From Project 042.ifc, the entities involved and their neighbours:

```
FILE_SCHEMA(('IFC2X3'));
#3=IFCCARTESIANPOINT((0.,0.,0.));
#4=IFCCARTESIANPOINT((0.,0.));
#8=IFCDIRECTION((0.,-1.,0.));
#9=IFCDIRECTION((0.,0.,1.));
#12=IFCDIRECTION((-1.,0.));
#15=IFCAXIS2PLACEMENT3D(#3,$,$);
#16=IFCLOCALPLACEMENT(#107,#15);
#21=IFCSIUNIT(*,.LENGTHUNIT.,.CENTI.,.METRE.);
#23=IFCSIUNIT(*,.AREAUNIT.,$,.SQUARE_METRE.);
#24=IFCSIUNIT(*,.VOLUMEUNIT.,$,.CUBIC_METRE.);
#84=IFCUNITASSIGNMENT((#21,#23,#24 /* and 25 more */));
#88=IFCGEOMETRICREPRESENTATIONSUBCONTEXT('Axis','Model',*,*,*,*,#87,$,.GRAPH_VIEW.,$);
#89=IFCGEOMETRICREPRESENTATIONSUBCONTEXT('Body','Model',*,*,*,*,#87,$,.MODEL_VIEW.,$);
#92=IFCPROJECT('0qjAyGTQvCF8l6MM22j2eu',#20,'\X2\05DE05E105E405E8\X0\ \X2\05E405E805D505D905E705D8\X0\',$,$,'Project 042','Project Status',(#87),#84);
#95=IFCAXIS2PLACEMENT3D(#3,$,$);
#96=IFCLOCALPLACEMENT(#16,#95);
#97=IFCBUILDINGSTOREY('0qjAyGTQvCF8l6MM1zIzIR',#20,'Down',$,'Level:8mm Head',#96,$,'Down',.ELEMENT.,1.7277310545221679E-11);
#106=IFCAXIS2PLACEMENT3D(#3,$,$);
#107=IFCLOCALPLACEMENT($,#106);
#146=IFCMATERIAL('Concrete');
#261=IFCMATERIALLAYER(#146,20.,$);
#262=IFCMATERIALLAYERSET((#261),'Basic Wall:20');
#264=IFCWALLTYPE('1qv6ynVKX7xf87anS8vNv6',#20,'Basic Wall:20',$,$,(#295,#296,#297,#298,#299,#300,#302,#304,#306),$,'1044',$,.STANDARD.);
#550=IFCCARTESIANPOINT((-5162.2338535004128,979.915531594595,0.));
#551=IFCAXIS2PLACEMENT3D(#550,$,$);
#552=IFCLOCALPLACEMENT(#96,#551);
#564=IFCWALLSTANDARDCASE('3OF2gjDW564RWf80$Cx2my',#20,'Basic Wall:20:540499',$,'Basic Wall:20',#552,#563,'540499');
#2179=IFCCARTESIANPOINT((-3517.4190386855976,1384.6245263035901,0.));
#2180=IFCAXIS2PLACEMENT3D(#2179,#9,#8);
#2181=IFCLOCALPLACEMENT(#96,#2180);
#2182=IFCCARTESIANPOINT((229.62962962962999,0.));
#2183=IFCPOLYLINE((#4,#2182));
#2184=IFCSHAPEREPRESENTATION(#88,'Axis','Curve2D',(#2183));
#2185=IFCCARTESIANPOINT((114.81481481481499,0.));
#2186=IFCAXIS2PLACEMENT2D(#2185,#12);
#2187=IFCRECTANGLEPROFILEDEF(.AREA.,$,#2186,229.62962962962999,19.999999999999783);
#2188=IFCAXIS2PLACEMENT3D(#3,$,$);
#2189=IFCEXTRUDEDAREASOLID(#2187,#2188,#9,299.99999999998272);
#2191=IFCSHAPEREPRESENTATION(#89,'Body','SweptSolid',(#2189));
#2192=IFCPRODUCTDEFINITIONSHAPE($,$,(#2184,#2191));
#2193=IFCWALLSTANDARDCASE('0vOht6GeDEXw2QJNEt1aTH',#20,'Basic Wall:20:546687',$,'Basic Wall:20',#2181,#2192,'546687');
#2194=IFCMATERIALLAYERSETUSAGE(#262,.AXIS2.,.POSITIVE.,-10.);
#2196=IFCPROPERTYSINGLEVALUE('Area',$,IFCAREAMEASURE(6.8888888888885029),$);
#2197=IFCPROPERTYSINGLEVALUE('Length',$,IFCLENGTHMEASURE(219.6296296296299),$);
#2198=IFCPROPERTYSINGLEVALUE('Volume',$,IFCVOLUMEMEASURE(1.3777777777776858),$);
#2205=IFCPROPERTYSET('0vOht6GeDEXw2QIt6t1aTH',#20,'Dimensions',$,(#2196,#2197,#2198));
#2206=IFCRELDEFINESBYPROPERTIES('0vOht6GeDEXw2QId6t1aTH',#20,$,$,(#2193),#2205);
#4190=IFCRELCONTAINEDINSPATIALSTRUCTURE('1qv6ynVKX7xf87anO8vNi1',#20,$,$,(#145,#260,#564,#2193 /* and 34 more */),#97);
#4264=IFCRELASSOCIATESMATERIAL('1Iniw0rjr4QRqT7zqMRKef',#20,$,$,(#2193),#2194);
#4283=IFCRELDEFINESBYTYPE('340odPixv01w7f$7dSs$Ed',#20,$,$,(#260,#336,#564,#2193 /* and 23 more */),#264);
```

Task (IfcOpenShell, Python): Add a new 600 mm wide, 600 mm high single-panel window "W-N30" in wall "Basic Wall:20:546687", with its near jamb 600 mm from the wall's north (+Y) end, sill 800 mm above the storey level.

```python
import numpy as np
import ifcopenshell
import ifcopenshell.api.feature
import ifcopenshell.api.geometry
import ifcopenshell.api.pset
import ifcopenshell.api.root
import ifcopenshell.api.spatial
import ifcopenshell.api.type
import ifcopenshell.geom
import ifcopenshell.util.element
import ifcopenshell.util.placement
import ifcopenshell.util.representation
import ifcopenshell.util.shape
import ifcopenshell.util.unit

model = ifcopenshell.open("Project 042.ifc")
unit_scale = ifcopenshell.util.unit.calculate_unit_scale(model)
area_scale = ifcopenshell.util.unit.calculate_unit_scale(model, "AREAUNIT")
volume_scale = ifcopenshell.util.unit.calculate_unit_scale(model, "VOLUMEUNIT")
settings = ifcopenshell.geom.settings()


def volume(element):
    """Net volume in cubic metres, openings subtracted."""
    shape = ifcopenshell.geom.create_shape(settings, element)
    return ifcopenshell.util.shape.get_volume(shape.geometry)


wall = model.by_id(2193)
storey = ifcopenshell.util.element.get_container(wall, ifc_class="IfcBuildingStorey")
context = ifcopenshell.util.representation.get_context(model, "Model", "Body", "MODEL_VIEW")
before = volume(wall)

width, height, from_end, sill = 0.6, 0.6, 0.6, 0.8  # metres

# The wall runs along its own X axis, and the end named is its -X end.
wall_shape = ifcopenshell.geom.create_shape(settings, wall)
x, y, z = ifcopenshell.util.shape.get_vertices(wall_shape.geometry).T
start = x.min() + from_end
face, thickness = float(y.min()), float(y.max() - y.min())
wall_matrix = ifcopenshell.util.placement.get_local_placement(wall.ObjectPlacement)
level = ifcopenshell.util.placement.get_local_placement(storey.ObjectPlacement)[2, 3]


def in_wall(x, y):
    """Placement at x, y metres in the wall's axes, at sill height."""
    matrix = wall_matrix.copy()
    matrix[:, 3] = wall_matrix @ np.array([x / unit_scale, y / unit_scale, 0.0, 1.0])
    matrix[2, 3] = level + sill / unit_scale
    return matrix


# Opening: a box that overshoots both wall faces by 50 mm.
opening = ifcopenshell.api.root.create_entity(model, ifc_class="IfcOpeningElement")
box = ifcopenshell.api.geometry.add_wall_representation(
    model, context=context, length=width, height=height, thickness=thickness + 0.1
)
ifcopenshell.api.geometry.assign_representation(model, product=opening, representation=box)
ifcopenshell.api.geometry.edit_object_placement(model, product=opening, matrix=in_wall(start, face - 0.05), is_si=False)
ifcopenshell.api.feature.add_feature(model, feature=opening, element=wall)

window = ifcopenshell.api.root.create_entity(model, ifc_class="IfcWindow", name="W-N30")
window.OverallWidth, window.OverallHeight = width / unit_scale, height / unit_scale
body = ifcopenshell.api.geometry.add_window_representation(
    model,
    context=context,
    overall_width=window.OverallWidth,
    overall_height=window.OverallHeight,
    partition_type="SINGLE_PANEL",
)
ifcopenshell.api.geometry.assign_representation(model, product=window, representation=body)
ifcopenshell.api.spatial.assign_container(model, products=[window], relating_structure=storey)
fills = ifcopenshell.api.feature.add_filling(model, opening=opening, element=window)
fills.OwnerHistory = window.OwnerHistory  # required in IFC2X3

# IFC2X3 keeps the operation on the window style.
style = ifcopenshell.api.root.create_entity(model, ifc_class="IfcWindowStyle", name="W-N30")
style.OperationType, style.ConstructionType = "SINGLE_PANEL", "NOTDEFINED"
style.ParameterTakesPrecedence = style.Sizeable = False
ifcopenshell.api.type.assign_type(model, related_objects=[window], relating_type=style)

# Centre the window in the wall's thickness.
ifcopenshell.api.geometry.edit_object_placement(model, product=window, matrix=in_wall(start, face), is_si=False)
window_shape = ifcopenshell.geom.create_shape(settings, window)
depth = ifcopenshell.util.shape.get_vertices(window_shape.geometry)[:, 1]
offset = face + thickness / 2 - (depth.min() + depth.max()) / 2
ifcopenshell.api.geometry.edit_object_placement(model, product=window, matrix=in_wall(start, offset), is_si=False)

after = volume(wall)

# Update the wall's stored quantities.
pset = model.by_id(ifcopenshell.util.element.get_pset(wall, "Dimensions", should_inherit=False)["id"])
ifcopenshell.api.pset.edit_pset(model, pset=pset, properties={
    "Area": model.create_entity("IfcAreaMeasure", after / thickness / area_scale),
    "Volume": model.create_entity("IfcVolumeMeasure", after / volume_scale),
})

print(f"wall volume {before:.3f} -> {after:.3f} m3")

model.write("Project 042_edited.ifc")
```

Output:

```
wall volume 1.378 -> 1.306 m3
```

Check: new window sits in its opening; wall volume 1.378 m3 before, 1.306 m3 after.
